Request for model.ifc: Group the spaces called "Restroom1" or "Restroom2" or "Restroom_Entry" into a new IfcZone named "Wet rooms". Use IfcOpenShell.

First a look at what the model holds.

```python
import ifcopenshell

model = ifcopenshell.open("model.ifc")
print(model.schema)
seen = {}
for space in model.by_type("IfcSpace"):
    seen[space.LongName] = seen.get(space.LongName, 0) + 1
for name, count in sorted(seen.items(), key=str):
    print(count, "x", name)
print("zones:", [z.Name for z in model.by_type("IfcZone")][:20])
```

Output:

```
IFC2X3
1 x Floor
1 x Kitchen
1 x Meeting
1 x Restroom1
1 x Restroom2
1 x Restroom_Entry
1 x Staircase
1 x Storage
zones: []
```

```python
import ifcopenshell
import ifcopenshell.api.group
import ifcopenshell.api.root

model = ifcopenshell.open("model.ifc")

names = {"Restroom1", "Restroom2", "Restroom_Entry"}
spaces = [s for s in model.by_type("IfcSpace") if s.LongName in names]

zone = ifcopenshell.api.root.create_entity(model, ifc_class="IfcZone", name="Wet rooms")
ifcopenshell.api.group.assign_group(model, products=spaces, group=zone)
print(len(spaces), "spaces in", zone.Name)

model.write("model-out.ifc")
```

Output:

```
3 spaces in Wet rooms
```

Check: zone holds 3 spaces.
